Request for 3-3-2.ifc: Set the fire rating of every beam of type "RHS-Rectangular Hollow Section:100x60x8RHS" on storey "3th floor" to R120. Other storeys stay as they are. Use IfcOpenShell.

First a look at what the model holds.

```python
import ifcopenshell
import ifcopenshell.util.element

model = ifcopenshell.open("3-3-2.ifc")
print(model.schema)
storey = next(s for s in model.by_type("IfcBuildingStorey") if s.Name == "3th floor")
beams = [e for e in ifcopenshell.util.element.get_decomposition(storey) if e.is_a("IfcBeam")]
seen = {}
for e in beams:
    element_type = ifcopenshell.util.element.get_type(e)
    key = (element_type.Name if element_type != e and element_type else None, ifcopenshell.util.element.get_pset(e, "Pset_BeamCommon", "FireRating"))
    seen[key] = seen.get(key, 0) + 1
for (name, value), count in sorted(seen.items(), key=str):
    print(count, "x", name, "|", value)
```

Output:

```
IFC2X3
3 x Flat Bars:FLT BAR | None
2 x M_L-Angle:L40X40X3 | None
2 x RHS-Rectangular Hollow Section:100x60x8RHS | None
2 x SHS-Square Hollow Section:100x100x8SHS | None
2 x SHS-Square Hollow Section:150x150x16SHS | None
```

```python
import ifcopenshell
import ifcopenshell.api.pset
import ifcopenshell.util.element

model = ifcopenshell.open("3-3-2.ifc")

storey = next(s for s in model.by_type("IfcBuildingStorey") if s.Name == "3th floor")
beams = [e for e in ifcopenshell.util.element.get_decomposition(storey) if e.is_a("IfcBeam")]

count = 0
for e in beams:
    element_type = ifcopenshell.util.element.get_type(e)
    if element_type in (None, e) or element_type.Name != "RHS-Rectangular Hollow Section:100x60x8RHS":
        continue
    # add_pset returns the element's existing set when there is one.
    pset = ifcopenshell.api.pset.add_pset(model, product=e, name="Pset_BeamCommon")
    ifcopenshell.api.pset.edit_pset(model, pset=pset, properties={"FireRating": "R120"})
    count += 1

print(count, "beams updated")

model.write("3-3-2_edited.ifc")
```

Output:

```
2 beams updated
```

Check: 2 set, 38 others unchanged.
